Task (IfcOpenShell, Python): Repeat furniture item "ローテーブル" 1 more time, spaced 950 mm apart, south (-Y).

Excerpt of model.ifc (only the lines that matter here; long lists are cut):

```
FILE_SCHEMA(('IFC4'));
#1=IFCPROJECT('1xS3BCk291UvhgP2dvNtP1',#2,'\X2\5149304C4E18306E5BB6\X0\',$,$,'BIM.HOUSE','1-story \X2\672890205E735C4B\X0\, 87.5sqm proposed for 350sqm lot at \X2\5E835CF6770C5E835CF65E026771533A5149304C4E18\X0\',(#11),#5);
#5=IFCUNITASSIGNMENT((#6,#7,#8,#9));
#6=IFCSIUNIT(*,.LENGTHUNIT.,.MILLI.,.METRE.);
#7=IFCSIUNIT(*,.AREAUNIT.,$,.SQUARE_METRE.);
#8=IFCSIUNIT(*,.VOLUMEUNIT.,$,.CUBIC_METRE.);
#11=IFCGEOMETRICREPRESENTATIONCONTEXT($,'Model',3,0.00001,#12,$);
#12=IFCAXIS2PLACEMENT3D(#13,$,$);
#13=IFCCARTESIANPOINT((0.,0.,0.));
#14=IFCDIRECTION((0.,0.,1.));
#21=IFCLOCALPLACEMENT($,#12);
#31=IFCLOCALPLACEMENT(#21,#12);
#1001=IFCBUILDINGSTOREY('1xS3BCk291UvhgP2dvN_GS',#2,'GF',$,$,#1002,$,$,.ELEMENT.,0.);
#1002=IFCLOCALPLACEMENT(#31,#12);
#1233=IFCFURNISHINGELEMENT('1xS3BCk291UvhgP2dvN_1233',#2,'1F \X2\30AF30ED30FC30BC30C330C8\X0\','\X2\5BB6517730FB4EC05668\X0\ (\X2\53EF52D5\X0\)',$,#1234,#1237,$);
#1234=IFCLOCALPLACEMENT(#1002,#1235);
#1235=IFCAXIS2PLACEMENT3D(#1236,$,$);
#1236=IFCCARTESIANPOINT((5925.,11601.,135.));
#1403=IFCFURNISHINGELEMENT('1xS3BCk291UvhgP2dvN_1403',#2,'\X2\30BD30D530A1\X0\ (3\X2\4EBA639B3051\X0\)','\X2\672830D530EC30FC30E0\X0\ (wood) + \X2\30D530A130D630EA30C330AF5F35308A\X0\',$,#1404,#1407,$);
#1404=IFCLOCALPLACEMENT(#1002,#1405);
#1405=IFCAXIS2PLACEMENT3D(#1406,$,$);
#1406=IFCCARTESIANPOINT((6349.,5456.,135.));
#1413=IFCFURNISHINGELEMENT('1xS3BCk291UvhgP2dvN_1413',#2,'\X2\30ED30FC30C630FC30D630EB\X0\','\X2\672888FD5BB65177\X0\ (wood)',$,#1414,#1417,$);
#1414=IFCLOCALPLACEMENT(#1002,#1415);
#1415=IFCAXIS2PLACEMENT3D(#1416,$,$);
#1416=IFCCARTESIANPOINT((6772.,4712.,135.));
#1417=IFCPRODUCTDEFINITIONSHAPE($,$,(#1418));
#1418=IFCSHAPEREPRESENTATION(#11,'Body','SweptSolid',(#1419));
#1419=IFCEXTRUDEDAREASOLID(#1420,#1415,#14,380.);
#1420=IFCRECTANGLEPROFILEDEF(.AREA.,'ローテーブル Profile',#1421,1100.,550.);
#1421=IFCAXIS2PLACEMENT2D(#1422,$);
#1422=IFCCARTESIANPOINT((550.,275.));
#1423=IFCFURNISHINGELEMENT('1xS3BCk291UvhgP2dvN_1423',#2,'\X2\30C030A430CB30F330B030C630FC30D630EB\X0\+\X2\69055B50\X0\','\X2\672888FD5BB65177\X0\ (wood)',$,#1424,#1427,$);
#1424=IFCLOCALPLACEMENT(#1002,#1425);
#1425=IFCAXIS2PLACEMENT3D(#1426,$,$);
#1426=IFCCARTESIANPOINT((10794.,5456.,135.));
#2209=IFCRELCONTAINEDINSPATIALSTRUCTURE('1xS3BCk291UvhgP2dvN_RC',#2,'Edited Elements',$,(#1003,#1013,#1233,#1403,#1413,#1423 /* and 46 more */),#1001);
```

```python
import numpy as np
import ifcopenshell
import ifcopenshell.api.geometry
import ifcopenshell.api.root
import ifcopenshell.util.element
import ifcopenshell.util.placement
import ifcopenshell.util.unit

model = ifcopenshell.open("model.ifc")
unit_scale = ifcopenshell.util.unit.calculate_unit_scale(model)


def reuse_history(source, copy):
    """copy_class also copies each property set's owner history, people and application; keep the originals."""
    for rel in copy.IsDefinedBy:
        if rel.is_a("IfcRelDefinesByProperties") and (history := rel.RelatingPropertyDefinition.OwnerHistory):
            rel.RelatingPropertyDefinition.OwnerHistory = source.OwnerHistory
            ifcopenshell.util.element.remove_deep2(model, history)


source = model.by_guid("1xS3BCk291UvhgP2dvN_1413")
base = ifcopenshell.util.placement.get_local_placement(source.ObjectPlacement)
step = np.array([0.0, -1.0, 0.0]) * 0.95 / unit_scale

for i in range(1, 2):
    copy = ifcopenshell.api.root.copy_class(model, product=source)
    copy.Representation = ifcopenshell.util.element.copy_deep(
        model, source.Representation, exclude=["IfcGeometricRepresentationContext", "IfcRepresentationMap"]
    )
    reuse_history(source, copy)
    matrix = base.copy()
    matrix[:3, 3] += i * step
    print("added at", matrix[:3, 3].round(3) + 0.0)
    ifcopenshell.api.geometry.edit_object_placement(model, product=copy, matrix=matrix, is_si=False)

model.write("model_updated.ifc")
```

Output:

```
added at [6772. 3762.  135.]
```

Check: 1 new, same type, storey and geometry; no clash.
